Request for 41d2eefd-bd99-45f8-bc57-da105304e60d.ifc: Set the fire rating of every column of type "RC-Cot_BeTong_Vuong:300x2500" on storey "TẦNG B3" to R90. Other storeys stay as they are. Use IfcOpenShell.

First a look at what the model holds.

```python
import ifcopenshell
import ifcopenshell.util.element

model = ifcopenshell.open("41d2eefd-bd99-45f8-bc57-da105304e60d.ifc")
print(model.schema)
storey = next(s for s in model.by_type("IfcBuildingStorey") if s.Name == "TẦNG B3")
columns = [e for e in ifcopenshell.util.element.get_decomposition(storey) if e.is_a("IfcColumn")]
seen = {}
for e in columns:
    element_type = ifcopenshell.util.element.get_type(e)
    key = (element_type.Name if element_type != e and element_type else None, ifcopenshell.util.element.get_pset(e, "Pset_ColumnCommon", "FireRating"))
    seen[key] = seen.get(key, 0) + 1
for (name, value), count in sorted(seen.items(), key=str):
    print(count, "x", name, "|", value)
```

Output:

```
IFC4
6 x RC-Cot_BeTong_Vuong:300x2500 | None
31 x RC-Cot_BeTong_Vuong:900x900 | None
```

```python
import ifcopenshell
import ifcopenshell.api.pset
import ifcopenshell.util.element

model = ifcopenshell.open("41d2eefd-bd99-45f8-bc57-da105304e60d.ifc")

storey = next(s for s in model.by_type("IfcBuildingStorey") if s.Name == "TẦNG B3")
columns = [e for e in ifcopenshell.util.element.get_decomposition(storey) if e.is_a("IfcColumn")]

count = 0
for e in columns:
    element_type = ifcopenshell.util.element.get_type(e)
    if element_type in (None, e) or element_type.Name != "RC-Cot_BeTong_Vuong:300x2500":
        continue
    # add_pset returns the element's existing set when there is one.
    pset = ifcopenshell.api.pset.add_pset(model, product=e, name="Pset_ColumnCommon")
    ifcopenshell.api.pset.edit_pset(model, pset=pset, properties={"FireRating": "R90"})
    count += 1

print(count, "columns updated")

model.write("41d2eefd-bd99-45f8-bc57-da105304e60d_v2.ifc")
```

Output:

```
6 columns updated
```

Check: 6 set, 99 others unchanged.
